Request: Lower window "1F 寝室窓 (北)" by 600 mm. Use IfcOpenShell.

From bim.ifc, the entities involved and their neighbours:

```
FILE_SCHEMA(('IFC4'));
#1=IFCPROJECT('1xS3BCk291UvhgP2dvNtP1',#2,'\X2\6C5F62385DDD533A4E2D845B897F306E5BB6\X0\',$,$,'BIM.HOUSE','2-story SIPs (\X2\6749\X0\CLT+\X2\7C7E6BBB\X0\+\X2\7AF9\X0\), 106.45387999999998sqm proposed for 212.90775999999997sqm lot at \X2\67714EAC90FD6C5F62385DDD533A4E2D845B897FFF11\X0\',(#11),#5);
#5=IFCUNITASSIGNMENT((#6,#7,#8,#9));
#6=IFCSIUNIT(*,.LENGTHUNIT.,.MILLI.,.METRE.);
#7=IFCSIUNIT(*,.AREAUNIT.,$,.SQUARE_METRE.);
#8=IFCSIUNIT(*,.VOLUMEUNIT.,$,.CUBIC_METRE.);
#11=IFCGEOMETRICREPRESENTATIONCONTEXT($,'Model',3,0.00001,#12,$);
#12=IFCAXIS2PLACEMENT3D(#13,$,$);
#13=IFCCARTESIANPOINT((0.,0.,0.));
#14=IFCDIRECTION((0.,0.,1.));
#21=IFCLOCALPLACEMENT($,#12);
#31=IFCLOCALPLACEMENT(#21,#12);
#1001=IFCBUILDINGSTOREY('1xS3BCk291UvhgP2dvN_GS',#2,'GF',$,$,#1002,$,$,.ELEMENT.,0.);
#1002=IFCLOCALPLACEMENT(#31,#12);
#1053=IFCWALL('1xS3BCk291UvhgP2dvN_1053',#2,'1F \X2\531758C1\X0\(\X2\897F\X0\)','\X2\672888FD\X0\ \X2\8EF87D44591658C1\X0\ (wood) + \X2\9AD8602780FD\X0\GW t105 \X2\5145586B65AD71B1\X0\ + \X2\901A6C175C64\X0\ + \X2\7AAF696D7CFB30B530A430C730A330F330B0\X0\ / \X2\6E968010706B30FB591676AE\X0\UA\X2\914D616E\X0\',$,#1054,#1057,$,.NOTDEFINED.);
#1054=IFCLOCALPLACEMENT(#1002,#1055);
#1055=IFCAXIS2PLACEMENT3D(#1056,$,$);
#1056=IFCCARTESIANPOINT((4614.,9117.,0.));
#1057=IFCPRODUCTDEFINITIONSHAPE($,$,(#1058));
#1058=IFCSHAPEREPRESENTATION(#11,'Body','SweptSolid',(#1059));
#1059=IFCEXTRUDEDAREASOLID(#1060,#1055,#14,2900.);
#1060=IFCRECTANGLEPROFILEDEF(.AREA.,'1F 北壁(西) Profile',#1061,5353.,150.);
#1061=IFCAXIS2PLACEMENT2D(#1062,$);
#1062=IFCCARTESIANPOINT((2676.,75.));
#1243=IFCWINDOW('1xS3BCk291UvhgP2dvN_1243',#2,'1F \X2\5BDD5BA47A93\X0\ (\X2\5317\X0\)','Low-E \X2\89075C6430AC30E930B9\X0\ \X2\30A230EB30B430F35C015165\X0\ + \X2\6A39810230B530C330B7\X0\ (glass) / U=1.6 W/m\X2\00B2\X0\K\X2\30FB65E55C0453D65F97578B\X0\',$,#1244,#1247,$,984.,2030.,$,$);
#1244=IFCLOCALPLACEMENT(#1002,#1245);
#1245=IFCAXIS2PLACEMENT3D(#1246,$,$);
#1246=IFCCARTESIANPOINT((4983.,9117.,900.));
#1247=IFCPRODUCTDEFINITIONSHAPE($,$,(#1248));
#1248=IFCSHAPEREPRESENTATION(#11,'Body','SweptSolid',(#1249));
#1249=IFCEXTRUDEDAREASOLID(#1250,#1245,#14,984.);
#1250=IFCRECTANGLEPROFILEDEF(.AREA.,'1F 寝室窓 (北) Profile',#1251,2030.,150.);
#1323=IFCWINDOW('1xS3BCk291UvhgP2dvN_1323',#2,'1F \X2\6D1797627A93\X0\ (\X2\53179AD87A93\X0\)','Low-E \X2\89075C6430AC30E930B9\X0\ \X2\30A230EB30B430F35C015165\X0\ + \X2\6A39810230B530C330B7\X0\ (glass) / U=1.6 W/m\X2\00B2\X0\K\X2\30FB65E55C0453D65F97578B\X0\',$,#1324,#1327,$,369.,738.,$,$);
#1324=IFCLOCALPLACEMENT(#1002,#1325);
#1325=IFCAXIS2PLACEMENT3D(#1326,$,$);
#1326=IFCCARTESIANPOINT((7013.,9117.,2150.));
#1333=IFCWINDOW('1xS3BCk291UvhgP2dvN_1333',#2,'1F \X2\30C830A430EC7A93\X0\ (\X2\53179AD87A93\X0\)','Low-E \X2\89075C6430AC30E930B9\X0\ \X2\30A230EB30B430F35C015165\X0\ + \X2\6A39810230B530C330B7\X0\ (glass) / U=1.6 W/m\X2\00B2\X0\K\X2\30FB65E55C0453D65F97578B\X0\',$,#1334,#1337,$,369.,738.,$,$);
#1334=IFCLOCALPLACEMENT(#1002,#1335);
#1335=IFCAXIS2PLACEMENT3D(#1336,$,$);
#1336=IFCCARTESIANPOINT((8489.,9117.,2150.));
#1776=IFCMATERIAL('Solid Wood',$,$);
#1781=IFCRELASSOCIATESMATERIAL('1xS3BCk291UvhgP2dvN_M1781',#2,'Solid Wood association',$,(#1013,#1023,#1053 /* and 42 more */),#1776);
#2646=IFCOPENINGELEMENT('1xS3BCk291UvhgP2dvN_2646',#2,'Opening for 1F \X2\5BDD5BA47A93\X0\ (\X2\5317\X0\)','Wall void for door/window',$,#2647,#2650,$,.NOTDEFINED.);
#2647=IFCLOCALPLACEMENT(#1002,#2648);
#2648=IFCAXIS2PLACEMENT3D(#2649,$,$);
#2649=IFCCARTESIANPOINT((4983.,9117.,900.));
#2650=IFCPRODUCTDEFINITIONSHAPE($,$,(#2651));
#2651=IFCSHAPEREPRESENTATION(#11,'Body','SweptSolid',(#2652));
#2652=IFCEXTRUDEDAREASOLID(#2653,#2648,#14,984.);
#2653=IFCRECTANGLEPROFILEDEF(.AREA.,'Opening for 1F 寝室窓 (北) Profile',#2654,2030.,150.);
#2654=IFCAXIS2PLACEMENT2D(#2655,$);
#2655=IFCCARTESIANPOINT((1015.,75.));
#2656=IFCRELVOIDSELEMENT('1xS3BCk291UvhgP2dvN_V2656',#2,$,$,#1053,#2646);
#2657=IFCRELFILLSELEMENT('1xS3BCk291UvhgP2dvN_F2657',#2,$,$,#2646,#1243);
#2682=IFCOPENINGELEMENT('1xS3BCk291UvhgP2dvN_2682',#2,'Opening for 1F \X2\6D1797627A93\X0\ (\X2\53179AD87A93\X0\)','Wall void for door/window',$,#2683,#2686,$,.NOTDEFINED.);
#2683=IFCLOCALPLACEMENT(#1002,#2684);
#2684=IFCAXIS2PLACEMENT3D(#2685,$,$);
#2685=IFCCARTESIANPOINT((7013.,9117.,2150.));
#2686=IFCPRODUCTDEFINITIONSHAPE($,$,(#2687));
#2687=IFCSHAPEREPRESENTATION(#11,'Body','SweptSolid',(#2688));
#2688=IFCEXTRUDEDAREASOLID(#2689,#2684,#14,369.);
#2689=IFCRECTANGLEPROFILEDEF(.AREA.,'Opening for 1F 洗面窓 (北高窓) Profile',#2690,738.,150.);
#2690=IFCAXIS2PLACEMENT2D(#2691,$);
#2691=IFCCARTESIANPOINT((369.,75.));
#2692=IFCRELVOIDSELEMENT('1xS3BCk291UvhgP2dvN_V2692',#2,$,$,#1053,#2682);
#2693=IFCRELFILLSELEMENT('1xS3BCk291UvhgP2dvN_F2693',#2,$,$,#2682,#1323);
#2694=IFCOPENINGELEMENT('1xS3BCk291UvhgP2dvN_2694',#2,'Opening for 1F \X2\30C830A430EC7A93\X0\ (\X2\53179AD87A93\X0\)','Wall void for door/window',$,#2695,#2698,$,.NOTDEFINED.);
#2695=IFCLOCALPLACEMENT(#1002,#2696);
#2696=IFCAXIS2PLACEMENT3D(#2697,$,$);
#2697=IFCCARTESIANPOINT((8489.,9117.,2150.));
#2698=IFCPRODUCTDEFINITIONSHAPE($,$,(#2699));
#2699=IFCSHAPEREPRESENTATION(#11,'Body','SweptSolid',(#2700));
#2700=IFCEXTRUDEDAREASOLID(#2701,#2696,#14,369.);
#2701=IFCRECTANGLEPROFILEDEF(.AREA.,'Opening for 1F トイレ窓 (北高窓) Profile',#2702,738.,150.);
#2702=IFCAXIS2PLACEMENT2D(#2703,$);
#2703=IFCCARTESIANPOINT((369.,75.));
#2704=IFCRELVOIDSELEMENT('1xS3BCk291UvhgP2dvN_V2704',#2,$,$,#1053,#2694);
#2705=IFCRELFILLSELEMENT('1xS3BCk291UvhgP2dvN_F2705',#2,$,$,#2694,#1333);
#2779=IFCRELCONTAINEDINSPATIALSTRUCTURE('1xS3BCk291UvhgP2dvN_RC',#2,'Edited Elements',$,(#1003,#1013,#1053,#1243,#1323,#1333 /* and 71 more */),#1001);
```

```python
import numpy as np
import ifcopenshell
import ifcopenshell.api.geometry
import ifcopenshell.util.placement
import ifcopenshell.util.unit

model = ifcopenshell.open("bim.ifc")
unit_scale = ifcopenshell.util.unit.calculate_unit_scale(model)

window = model.by_guid("1xS3BCk291UvhgP2dvN_1243")
opening = window.FillsVoids[0].RelatingOpeningElement
dz = -0.6 / unit_scale

shift = np.array([0.0, 0.0, dz])
# The window is not placed relative to its opening, so move both.
for product in (opening, window):
    matrix = ifcopenshell.util.placement.get_local_placement(product.ObjectPlacement)
    matrix[:3, 3] += shift
    ifcopenshell.api.geometry.edit_object_placement(model, product=product, matrix=matrix, is_si=False)

print(f"moved by {dz * unit_scale:+.3f} m")

model.write("bim_updated.ifc")
```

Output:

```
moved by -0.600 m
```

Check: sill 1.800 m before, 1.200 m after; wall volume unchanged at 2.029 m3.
